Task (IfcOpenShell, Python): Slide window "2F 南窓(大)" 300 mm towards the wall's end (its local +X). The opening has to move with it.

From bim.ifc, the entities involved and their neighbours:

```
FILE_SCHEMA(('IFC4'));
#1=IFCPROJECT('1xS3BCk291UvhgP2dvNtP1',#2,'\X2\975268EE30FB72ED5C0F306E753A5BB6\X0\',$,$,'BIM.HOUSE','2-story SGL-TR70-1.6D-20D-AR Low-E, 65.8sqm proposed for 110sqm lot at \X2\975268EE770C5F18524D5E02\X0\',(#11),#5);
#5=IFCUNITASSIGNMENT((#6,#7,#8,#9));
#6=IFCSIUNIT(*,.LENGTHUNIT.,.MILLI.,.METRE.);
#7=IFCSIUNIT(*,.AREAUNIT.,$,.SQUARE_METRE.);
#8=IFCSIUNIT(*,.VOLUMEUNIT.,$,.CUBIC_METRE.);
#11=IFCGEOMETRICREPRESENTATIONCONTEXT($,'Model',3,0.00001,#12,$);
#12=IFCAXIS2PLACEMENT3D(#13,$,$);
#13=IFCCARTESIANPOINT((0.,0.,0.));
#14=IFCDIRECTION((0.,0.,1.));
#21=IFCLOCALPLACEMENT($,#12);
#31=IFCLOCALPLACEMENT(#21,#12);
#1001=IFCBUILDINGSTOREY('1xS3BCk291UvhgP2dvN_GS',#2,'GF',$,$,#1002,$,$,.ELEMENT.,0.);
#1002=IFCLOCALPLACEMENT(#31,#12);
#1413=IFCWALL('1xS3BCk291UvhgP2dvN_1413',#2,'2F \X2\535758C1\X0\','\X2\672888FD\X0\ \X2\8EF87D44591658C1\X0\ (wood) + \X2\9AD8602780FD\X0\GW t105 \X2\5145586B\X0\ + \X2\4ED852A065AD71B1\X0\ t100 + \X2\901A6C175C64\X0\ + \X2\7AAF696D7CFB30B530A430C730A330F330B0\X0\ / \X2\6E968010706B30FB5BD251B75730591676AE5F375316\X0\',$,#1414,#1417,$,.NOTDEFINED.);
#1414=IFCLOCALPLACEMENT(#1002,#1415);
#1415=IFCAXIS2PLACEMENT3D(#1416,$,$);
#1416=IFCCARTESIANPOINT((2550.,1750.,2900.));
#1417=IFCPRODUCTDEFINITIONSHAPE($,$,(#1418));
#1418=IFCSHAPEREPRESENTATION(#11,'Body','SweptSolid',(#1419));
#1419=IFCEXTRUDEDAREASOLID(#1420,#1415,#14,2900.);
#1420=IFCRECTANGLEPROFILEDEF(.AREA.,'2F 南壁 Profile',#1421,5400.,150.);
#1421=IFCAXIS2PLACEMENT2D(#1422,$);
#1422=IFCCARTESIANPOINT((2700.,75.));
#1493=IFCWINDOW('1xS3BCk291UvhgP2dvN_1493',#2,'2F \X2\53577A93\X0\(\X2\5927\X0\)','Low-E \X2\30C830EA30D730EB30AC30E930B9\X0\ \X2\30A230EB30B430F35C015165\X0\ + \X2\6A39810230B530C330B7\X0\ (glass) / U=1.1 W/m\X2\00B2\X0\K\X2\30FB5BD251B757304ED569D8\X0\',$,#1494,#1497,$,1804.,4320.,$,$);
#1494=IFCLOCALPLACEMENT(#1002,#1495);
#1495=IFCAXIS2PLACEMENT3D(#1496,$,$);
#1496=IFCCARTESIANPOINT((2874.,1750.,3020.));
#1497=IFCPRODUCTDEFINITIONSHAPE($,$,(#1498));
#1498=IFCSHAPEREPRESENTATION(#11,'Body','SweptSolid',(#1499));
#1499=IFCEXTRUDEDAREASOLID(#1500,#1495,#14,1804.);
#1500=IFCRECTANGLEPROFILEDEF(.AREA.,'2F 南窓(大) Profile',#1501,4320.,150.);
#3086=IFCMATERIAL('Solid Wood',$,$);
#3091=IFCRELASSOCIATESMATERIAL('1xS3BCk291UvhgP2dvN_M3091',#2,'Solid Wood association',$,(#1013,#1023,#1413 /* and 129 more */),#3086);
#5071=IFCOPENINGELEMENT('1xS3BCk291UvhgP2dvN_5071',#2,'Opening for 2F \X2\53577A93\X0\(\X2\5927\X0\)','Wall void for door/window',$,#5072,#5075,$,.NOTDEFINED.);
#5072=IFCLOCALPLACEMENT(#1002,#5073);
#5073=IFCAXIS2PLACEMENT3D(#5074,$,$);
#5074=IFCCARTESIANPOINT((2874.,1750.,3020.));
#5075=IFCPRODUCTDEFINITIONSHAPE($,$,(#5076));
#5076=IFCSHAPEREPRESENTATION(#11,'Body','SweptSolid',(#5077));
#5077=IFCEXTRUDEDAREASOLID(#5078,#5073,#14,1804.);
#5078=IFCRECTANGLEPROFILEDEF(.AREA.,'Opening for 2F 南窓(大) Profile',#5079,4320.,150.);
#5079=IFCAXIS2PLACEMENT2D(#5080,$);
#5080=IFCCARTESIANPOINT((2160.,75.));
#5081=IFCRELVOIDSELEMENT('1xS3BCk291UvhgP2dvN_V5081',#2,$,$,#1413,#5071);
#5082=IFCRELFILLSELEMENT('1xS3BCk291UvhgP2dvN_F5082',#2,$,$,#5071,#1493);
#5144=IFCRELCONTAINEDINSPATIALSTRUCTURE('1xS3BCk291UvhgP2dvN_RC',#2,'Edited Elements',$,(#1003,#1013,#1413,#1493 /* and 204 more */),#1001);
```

```python
import ifcopenshell
import ifcopenshell.api.geometry
import ifcopenshell.util.placement

model = ifcopenshell.open("bim.ifc")

window = model.by_guid("1xS3BCk291UvhgP2dvN_1493")
opening = window.FillsVoids[0].RelatingOpeningElement
wall = opening.VoidsElements[0].RelatingBuildingElement

wall_matrix = ifcopenshell.util.placement.get_local_placement(wall.ObjectPlacement)
shift = wall_matrix[:3, 0] * 300.0
before = ifcopenshell.util.placement.get_local_placement(window.ObjectPlacement)[:3, 3].copy()

# The window is not placed relative to its opening, so move both.
for product in (opening, window):
    matrix = ifcopenshell.util.placement.get_local_placement(product.ObjectPlacement)
    matrix[:3, 3] += shift
    ifcopenshell.api.geometry.edit_object_placement(model, product=product, matrix=matrix, is_si=False)

after = ifcopenshell.util.placement.get_local_placement(window.ObjectPlacement)[:3, 3]
print("window moved by", (after - before).round(3) + 0.0)

model.write("bim_rev.ifc")
```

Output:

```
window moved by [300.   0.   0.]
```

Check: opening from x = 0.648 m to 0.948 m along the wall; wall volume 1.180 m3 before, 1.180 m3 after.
